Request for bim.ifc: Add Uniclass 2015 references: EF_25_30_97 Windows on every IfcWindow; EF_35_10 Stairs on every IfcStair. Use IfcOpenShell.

First a look at what the model holds.

```python
import ifcopenshell

model = ifcopenshell.open("bim.ifc")
print(model.schema)
print("classifications:", [c.Name for c in model.by_type("IfcClassification")])
for ifc_class in ("IfcDoor", "IfcRoof", "IfcStair", "IfcWall", "IfcWindow"):
    print(ifc_class, len(model.by_type(ifc_class)))
```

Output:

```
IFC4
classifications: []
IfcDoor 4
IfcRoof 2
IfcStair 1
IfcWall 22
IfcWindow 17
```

```python
import ifcopenshell
import ifcopenshell.api.classification

model = ifcopenshell.open("bim.ifc")

system = ifcopenshell.api.classification.add_classification(model, classification="Uniclass 2015")

codes = {
    "IfcWindow": ("EF_25_30_97", "Windows"),
    "IfcStair": ("EF_35_10", "Stairs"),
}
for ifc_class, (code, name) in codes.items():
    products = model.by_type(ifc_class)
    ifcopenshell.api.classification.add_reference(
        model, products=products, classification=system, identification=code, name=name
    )
    print(code, len(products))

model.write("bim-out.ifc")
```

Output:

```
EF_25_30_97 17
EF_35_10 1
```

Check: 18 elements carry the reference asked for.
